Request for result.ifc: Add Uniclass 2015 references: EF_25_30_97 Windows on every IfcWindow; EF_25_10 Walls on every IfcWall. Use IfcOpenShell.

First a look at what the model holds.

```python
import ifcopenshell

model = ifcopenshell.open("result.ifc")
print(model.schema)
print("classifications:", [c.Name for c in model.by_type("IfcClassification")])
for ifc_class in ("IfcDoor", "IfcRoof", "IfcStair", "IfcWall", "IfcWindow"):
    print(ifc_class, len(model.by_type(ifc_class)))
```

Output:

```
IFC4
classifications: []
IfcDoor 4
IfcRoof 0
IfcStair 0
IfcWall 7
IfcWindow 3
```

```python
import ifcopenshell
import ifcopenshell.api.classification

model = ifcopenshell.open("result.ifc")

system = ifcopenshell.api.classification.add_classification(model, classification="Uniclass 2015")

codes = {
    "IfcWindow": ("EF_25_30_97", "Windows"),
    "IfcWall": ("EF_25_10", "Walls"),
}
for ifc_class, (code, name) in codes.items():
    products = model.by_type(ifc_class)
    ifcopenshell.api.classification.add_reference(
        model, products=products, classification=system, identification=code, name=name
    )
    print(code, len(products))

model.write("result_v2.ifc")
```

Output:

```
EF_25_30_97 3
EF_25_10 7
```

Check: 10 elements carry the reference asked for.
